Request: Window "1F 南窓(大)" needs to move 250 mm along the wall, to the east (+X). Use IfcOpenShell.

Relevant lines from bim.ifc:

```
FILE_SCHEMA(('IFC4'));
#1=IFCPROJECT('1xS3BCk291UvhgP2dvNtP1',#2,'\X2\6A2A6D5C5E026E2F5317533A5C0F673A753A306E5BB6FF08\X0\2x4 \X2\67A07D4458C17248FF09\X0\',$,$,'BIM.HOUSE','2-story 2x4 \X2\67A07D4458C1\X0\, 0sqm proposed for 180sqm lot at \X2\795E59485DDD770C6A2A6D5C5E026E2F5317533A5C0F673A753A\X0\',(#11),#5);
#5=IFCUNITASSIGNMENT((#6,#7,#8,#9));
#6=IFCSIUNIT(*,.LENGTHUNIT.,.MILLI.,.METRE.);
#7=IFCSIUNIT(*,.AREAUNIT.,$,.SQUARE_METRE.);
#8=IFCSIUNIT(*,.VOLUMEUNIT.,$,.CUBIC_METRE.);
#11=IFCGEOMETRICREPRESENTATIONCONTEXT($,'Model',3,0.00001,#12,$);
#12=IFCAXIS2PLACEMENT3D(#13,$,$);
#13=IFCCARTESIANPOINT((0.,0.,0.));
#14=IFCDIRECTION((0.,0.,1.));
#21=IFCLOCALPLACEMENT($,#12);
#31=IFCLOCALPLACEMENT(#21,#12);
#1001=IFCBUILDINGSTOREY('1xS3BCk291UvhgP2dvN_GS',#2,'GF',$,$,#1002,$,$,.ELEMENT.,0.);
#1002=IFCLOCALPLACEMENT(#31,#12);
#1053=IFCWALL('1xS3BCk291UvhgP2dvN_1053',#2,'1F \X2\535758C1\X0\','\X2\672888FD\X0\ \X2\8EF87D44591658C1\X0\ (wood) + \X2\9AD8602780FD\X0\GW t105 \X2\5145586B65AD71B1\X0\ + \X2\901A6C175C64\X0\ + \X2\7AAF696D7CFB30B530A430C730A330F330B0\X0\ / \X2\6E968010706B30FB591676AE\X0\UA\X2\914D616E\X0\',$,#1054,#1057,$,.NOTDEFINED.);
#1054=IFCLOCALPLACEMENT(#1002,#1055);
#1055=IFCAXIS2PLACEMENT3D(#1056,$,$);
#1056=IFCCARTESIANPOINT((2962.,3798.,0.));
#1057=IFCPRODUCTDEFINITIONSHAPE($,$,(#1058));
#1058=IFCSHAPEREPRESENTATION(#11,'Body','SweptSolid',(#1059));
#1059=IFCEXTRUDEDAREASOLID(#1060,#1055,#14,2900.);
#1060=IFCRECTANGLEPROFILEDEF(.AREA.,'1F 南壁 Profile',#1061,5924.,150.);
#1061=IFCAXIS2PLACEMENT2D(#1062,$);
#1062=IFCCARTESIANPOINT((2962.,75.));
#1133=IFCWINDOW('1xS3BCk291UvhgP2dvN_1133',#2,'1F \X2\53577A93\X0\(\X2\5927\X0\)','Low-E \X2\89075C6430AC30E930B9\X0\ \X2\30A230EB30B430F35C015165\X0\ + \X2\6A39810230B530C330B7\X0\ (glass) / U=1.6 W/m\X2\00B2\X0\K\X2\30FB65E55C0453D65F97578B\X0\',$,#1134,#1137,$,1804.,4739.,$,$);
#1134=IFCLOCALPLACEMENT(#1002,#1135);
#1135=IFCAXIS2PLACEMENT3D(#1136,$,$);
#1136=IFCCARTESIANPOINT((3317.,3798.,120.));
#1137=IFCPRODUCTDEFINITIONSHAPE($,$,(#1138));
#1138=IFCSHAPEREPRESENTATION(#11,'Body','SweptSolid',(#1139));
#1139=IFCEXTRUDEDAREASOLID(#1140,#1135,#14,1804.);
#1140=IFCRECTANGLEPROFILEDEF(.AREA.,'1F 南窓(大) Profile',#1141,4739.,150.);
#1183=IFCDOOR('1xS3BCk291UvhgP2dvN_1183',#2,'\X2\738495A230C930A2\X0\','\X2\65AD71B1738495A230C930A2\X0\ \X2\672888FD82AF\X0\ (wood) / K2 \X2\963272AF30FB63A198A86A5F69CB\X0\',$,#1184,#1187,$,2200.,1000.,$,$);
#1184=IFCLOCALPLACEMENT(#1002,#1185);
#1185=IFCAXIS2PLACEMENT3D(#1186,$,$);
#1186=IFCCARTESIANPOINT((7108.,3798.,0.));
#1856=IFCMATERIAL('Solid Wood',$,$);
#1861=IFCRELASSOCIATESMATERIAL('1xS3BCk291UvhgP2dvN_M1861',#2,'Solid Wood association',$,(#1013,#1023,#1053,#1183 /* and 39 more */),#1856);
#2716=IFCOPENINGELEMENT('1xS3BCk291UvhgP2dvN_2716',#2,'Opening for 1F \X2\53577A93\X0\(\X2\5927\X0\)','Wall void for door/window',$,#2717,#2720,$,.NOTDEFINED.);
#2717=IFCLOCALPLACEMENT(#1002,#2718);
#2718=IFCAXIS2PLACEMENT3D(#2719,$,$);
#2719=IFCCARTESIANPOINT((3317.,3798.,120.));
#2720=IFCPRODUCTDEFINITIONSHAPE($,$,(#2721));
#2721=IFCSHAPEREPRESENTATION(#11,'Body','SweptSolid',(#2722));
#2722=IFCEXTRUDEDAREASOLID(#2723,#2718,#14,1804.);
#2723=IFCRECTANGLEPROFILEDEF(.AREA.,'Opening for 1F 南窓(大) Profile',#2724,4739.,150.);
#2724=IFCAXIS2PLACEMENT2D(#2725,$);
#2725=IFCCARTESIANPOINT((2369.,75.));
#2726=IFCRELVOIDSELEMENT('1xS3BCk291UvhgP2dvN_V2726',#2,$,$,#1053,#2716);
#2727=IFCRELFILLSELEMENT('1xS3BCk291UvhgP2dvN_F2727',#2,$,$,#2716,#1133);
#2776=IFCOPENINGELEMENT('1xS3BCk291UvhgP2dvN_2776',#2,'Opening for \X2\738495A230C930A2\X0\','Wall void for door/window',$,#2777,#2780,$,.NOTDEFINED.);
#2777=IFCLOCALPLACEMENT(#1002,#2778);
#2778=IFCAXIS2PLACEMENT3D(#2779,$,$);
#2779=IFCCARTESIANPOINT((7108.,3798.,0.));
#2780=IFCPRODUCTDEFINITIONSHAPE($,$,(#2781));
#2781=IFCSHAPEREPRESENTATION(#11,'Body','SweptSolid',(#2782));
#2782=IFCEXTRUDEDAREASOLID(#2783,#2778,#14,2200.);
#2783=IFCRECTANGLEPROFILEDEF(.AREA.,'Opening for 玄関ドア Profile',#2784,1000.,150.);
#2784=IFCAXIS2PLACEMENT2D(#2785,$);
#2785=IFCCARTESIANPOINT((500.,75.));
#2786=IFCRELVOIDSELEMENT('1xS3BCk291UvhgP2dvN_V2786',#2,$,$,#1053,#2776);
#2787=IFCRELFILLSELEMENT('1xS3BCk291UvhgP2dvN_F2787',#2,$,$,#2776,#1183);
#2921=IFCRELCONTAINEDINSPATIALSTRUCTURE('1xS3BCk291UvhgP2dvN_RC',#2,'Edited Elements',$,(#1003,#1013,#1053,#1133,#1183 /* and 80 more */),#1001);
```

```python
import ifcopenshell
import ifcopenshell.api.geometry
import ifcopenshell.util.placement

model = ifcopenshell.open("bim.ifc")

window = model.by_id(1133)
opening = window.FillsVoids[0].RelatingOpeningElement
wall = opening.VoidsElements[0].RelatingBuildingElement

wall_matrix = ifcopenshell.util.placement.get_local_placement(wall.ObjectPlacement)
shift = wall_matrix[:3, 0] * 250.0
before = ifcopenshell.util.placement.get_local_placement(window.ObjectPlacement)[:3, 3].copy()

# The window is not placed relative to its opening, so move both.
for product in (opening, window):
    matrix = ifcopenshell.util.placement.get_local_placement(product.ObjectPlacement)
    matrix[:3, 3] += shift
    ifcopenshell.api.geometry.edit_object_placement(model, product=product, matrix=matrix, is_si=False)

after = ifcopenshell.util.placement.get_local_placement(window.ObjectPlacement)[:3, 3]
print("window moved by", (after - before).round(3) + 0.0)

model.write("bim_v2.ifc")
```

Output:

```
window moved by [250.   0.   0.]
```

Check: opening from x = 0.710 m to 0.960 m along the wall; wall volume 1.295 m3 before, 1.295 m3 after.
